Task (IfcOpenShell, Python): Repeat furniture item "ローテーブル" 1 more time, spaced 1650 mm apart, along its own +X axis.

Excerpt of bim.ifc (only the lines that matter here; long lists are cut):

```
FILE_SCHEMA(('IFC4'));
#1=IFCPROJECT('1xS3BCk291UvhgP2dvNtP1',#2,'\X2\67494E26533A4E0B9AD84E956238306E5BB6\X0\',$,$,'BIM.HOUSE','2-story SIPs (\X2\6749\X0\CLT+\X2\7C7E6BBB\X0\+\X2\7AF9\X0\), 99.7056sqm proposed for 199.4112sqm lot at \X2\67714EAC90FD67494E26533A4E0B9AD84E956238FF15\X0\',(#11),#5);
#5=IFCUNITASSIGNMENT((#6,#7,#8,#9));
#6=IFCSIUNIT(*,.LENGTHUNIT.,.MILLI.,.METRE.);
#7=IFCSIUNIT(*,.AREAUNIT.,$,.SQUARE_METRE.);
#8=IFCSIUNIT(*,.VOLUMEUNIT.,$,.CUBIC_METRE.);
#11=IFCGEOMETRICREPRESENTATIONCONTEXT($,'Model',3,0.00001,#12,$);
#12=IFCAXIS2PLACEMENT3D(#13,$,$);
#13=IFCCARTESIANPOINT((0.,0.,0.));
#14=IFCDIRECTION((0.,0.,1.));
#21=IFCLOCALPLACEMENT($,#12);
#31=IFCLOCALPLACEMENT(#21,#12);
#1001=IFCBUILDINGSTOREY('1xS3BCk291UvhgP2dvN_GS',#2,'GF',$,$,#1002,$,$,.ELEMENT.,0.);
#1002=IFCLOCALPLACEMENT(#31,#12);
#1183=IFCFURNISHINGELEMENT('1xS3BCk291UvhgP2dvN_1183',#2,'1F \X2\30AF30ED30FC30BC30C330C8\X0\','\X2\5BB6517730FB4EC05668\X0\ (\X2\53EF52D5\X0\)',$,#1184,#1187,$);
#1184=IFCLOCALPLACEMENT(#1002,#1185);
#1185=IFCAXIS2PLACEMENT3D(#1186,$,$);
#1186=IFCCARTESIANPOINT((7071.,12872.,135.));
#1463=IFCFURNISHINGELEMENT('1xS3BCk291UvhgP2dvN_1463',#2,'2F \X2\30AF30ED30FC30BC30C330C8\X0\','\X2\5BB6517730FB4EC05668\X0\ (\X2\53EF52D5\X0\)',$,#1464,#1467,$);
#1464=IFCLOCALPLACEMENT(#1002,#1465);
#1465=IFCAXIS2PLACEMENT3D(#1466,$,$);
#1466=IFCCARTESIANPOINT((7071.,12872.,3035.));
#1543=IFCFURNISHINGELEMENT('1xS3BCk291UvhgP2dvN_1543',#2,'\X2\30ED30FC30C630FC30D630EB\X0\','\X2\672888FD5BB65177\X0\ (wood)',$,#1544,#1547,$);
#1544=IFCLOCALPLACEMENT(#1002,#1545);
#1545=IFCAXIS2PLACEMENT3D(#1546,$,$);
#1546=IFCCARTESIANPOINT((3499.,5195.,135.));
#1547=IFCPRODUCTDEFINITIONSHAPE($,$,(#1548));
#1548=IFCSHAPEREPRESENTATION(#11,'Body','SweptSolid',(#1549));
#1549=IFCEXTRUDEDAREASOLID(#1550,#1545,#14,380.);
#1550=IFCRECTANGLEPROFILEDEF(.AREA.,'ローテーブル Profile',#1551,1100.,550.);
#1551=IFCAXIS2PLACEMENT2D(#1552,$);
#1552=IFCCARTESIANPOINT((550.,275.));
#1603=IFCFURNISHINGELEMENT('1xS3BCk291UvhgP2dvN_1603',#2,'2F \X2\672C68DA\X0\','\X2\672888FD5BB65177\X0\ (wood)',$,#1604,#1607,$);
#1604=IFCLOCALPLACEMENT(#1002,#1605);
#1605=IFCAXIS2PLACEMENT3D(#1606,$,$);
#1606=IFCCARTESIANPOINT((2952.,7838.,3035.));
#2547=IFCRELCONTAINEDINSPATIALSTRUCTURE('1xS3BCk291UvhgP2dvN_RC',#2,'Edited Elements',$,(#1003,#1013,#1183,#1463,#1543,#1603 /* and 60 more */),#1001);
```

```python
import ifcopenshell
import ifcopenshell.api.geometry
import ifcopenshell.api.root
import ifcopenshell.util.element
import ifcopenshell.util.placement
import ifcopenshell.util.unit

model = ifcopenshell.open("bim.ifc")
unit_scale = ifcopenshell.util.unit.calculate_unit_scale(model)


def reuse_history(source, copy):
    """copy_class also copies each property set's owner history, people and application; keep the originals."""
    for rel in copy.IsDefinedBy:
        if rel.is_a("IfcRelDefinesByProperties") and (history := rel.RelatingPropertyDefinition.OwnerHistory):
            rel.RelatingPropertyDefinition.OwnerHistory = source.OwnerHistory
            ifcopenshell.util.element.remove_deep2(model, history)


source = model.by_guid("1xS3BCk291UvhgP2dvN_1543")
base = ifcopenshell.util.placement.get_local_placement(source.ObjectPlacement)
step = base[:3, 0] * 1.65 / unit_scale

for i in range(1, 2):
    copy = ifcopenshell.api.root.copy_class(model, product=source)
    copy.Representation = ifcopenshell.util.element.copy_deep(
        model, source.Representation, exclude=["IfcGeometricRepresentationContext", "IfcRepresentationMap"]
    )
    reuse_history(source, copy)
    matrix = base.copy()
    matrix[:3, 3] += i * step
    print("added at", matrix[:3, 3].round(3) + 0.0)
    ifcopenshell.api.geometry.edit_object_placement(model, product=copy, matrix=matrix, is_si=False)

model.write("bim_edited.ifc")
```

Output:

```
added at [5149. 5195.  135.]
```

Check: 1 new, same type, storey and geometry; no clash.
